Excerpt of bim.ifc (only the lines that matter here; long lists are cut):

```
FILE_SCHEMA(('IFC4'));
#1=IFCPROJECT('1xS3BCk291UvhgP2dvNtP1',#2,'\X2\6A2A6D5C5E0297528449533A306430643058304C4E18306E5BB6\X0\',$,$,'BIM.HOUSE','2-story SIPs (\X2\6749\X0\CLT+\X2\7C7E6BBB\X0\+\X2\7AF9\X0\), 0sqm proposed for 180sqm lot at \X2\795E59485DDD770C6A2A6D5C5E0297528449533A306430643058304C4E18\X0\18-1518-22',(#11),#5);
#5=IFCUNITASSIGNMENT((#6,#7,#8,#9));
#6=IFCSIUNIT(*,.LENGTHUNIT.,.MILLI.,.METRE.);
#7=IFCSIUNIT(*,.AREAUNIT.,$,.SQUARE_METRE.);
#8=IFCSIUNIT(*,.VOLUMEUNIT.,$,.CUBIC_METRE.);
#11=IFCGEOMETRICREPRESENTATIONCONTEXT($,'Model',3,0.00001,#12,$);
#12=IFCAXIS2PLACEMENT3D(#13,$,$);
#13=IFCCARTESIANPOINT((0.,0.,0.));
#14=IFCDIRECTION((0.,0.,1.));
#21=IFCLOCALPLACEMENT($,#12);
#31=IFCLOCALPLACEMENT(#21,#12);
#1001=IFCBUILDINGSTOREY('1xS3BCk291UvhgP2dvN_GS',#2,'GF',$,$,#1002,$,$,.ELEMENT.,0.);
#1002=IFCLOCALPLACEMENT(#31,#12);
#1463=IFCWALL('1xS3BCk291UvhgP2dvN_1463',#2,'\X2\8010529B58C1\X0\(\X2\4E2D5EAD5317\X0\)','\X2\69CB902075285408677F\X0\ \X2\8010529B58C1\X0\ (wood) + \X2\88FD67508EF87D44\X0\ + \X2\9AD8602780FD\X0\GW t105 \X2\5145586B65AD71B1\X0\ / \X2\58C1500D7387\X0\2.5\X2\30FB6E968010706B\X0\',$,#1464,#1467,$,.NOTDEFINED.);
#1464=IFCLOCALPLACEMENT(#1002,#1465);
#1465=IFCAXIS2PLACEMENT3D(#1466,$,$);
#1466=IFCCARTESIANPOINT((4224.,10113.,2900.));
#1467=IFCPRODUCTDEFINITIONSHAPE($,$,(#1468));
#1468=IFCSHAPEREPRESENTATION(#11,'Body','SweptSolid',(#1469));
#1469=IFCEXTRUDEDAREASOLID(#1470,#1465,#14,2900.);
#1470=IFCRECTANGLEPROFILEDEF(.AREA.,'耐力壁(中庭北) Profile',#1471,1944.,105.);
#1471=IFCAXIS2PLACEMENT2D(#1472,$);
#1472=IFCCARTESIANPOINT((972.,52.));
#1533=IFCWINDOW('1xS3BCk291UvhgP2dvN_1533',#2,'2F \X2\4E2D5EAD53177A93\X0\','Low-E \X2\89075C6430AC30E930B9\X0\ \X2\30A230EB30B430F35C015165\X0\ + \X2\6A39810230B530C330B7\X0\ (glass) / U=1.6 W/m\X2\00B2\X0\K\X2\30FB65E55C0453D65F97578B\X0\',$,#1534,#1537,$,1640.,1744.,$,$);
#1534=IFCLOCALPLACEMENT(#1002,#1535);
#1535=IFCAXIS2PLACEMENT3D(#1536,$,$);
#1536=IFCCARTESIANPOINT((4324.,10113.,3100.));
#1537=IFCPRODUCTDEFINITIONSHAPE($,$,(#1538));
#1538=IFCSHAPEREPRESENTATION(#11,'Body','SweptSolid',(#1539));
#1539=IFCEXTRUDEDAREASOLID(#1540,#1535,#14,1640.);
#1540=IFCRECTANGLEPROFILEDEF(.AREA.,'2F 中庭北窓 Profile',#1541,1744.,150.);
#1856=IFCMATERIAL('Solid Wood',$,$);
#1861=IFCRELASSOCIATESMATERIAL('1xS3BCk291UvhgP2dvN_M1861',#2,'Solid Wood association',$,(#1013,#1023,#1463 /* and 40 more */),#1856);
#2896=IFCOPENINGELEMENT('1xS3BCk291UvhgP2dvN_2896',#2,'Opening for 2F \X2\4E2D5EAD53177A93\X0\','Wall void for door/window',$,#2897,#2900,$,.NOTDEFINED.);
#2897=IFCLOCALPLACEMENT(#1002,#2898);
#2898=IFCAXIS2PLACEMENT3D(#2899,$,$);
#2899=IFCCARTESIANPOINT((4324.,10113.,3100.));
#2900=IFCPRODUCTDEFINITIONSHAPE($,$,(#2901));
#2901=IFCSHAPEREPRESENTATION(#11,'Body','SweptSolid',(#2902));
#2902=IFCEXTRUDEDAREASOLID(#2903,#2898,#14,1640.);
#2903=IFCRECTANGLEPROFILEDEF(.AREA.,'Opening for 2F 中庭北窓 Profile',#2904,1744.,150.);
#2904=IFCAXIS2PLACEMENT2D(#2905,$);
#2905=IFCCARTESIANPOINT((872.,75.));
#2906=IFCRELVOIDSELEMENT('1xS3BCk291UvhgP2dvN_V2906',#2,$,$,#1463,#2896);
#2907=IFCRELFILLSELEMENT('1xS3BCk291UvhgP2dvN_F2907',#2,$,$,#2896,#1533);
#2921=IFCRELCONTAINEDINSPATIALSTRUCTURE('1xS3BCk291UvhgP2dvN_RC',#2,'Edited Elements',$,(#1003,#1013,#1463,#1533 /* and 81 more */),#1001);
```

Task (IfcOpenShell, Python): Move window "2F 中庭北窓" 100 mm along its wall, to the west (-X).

```python
import ifcopenshell
import ifcopenshell.api.geometry
import ifcopenshell.util.placement
import ifcopenshell.util.unit

model = ifcopenshell.open("bim.ifc")
unit_scale = ifcopenshell.util.unit.calculate_unit_scale(model)

window = model.by_guid("1xS3BCk291UvhgP2dvN_1533")
opening = window.FillsVoids[0].RelatingOpeningElement
wall = opening.VoidsElements[0].RelatingBuildingElement

wall_matrix = ifcopenshell.util.placement.get_local_placement(wall.ObjectPlacement)
shift = wall_matrix[:3, 0] * -0.1 / unit_scale
before = ifcopenshell.util.placement.get_local_placement(window.ObjectPlacement)[:3, 3].copy()

# The window is not placed relative to its opening, so move both.
for product in (opening, window):
    matrix = ifcopenshell.util.placement.get_local_placement(product.ObjectPlacement)
    matrix[:3, 3] += shift
    ifcopenshell.api.geometry.edit_object_placement(model, product=product, matrix=matrix, is_si=False)

after = ifcopenshell.util.placement.get_local_placement(window.ObjectPlacement)[:3, 3]
print("window moved by", (after - before).round(3) + 0.0)

model.write("bim_updated.ifc")
```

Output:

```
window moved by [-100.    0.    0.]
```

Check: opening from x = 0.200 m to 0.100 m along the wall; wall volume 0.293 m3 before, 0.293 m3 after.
